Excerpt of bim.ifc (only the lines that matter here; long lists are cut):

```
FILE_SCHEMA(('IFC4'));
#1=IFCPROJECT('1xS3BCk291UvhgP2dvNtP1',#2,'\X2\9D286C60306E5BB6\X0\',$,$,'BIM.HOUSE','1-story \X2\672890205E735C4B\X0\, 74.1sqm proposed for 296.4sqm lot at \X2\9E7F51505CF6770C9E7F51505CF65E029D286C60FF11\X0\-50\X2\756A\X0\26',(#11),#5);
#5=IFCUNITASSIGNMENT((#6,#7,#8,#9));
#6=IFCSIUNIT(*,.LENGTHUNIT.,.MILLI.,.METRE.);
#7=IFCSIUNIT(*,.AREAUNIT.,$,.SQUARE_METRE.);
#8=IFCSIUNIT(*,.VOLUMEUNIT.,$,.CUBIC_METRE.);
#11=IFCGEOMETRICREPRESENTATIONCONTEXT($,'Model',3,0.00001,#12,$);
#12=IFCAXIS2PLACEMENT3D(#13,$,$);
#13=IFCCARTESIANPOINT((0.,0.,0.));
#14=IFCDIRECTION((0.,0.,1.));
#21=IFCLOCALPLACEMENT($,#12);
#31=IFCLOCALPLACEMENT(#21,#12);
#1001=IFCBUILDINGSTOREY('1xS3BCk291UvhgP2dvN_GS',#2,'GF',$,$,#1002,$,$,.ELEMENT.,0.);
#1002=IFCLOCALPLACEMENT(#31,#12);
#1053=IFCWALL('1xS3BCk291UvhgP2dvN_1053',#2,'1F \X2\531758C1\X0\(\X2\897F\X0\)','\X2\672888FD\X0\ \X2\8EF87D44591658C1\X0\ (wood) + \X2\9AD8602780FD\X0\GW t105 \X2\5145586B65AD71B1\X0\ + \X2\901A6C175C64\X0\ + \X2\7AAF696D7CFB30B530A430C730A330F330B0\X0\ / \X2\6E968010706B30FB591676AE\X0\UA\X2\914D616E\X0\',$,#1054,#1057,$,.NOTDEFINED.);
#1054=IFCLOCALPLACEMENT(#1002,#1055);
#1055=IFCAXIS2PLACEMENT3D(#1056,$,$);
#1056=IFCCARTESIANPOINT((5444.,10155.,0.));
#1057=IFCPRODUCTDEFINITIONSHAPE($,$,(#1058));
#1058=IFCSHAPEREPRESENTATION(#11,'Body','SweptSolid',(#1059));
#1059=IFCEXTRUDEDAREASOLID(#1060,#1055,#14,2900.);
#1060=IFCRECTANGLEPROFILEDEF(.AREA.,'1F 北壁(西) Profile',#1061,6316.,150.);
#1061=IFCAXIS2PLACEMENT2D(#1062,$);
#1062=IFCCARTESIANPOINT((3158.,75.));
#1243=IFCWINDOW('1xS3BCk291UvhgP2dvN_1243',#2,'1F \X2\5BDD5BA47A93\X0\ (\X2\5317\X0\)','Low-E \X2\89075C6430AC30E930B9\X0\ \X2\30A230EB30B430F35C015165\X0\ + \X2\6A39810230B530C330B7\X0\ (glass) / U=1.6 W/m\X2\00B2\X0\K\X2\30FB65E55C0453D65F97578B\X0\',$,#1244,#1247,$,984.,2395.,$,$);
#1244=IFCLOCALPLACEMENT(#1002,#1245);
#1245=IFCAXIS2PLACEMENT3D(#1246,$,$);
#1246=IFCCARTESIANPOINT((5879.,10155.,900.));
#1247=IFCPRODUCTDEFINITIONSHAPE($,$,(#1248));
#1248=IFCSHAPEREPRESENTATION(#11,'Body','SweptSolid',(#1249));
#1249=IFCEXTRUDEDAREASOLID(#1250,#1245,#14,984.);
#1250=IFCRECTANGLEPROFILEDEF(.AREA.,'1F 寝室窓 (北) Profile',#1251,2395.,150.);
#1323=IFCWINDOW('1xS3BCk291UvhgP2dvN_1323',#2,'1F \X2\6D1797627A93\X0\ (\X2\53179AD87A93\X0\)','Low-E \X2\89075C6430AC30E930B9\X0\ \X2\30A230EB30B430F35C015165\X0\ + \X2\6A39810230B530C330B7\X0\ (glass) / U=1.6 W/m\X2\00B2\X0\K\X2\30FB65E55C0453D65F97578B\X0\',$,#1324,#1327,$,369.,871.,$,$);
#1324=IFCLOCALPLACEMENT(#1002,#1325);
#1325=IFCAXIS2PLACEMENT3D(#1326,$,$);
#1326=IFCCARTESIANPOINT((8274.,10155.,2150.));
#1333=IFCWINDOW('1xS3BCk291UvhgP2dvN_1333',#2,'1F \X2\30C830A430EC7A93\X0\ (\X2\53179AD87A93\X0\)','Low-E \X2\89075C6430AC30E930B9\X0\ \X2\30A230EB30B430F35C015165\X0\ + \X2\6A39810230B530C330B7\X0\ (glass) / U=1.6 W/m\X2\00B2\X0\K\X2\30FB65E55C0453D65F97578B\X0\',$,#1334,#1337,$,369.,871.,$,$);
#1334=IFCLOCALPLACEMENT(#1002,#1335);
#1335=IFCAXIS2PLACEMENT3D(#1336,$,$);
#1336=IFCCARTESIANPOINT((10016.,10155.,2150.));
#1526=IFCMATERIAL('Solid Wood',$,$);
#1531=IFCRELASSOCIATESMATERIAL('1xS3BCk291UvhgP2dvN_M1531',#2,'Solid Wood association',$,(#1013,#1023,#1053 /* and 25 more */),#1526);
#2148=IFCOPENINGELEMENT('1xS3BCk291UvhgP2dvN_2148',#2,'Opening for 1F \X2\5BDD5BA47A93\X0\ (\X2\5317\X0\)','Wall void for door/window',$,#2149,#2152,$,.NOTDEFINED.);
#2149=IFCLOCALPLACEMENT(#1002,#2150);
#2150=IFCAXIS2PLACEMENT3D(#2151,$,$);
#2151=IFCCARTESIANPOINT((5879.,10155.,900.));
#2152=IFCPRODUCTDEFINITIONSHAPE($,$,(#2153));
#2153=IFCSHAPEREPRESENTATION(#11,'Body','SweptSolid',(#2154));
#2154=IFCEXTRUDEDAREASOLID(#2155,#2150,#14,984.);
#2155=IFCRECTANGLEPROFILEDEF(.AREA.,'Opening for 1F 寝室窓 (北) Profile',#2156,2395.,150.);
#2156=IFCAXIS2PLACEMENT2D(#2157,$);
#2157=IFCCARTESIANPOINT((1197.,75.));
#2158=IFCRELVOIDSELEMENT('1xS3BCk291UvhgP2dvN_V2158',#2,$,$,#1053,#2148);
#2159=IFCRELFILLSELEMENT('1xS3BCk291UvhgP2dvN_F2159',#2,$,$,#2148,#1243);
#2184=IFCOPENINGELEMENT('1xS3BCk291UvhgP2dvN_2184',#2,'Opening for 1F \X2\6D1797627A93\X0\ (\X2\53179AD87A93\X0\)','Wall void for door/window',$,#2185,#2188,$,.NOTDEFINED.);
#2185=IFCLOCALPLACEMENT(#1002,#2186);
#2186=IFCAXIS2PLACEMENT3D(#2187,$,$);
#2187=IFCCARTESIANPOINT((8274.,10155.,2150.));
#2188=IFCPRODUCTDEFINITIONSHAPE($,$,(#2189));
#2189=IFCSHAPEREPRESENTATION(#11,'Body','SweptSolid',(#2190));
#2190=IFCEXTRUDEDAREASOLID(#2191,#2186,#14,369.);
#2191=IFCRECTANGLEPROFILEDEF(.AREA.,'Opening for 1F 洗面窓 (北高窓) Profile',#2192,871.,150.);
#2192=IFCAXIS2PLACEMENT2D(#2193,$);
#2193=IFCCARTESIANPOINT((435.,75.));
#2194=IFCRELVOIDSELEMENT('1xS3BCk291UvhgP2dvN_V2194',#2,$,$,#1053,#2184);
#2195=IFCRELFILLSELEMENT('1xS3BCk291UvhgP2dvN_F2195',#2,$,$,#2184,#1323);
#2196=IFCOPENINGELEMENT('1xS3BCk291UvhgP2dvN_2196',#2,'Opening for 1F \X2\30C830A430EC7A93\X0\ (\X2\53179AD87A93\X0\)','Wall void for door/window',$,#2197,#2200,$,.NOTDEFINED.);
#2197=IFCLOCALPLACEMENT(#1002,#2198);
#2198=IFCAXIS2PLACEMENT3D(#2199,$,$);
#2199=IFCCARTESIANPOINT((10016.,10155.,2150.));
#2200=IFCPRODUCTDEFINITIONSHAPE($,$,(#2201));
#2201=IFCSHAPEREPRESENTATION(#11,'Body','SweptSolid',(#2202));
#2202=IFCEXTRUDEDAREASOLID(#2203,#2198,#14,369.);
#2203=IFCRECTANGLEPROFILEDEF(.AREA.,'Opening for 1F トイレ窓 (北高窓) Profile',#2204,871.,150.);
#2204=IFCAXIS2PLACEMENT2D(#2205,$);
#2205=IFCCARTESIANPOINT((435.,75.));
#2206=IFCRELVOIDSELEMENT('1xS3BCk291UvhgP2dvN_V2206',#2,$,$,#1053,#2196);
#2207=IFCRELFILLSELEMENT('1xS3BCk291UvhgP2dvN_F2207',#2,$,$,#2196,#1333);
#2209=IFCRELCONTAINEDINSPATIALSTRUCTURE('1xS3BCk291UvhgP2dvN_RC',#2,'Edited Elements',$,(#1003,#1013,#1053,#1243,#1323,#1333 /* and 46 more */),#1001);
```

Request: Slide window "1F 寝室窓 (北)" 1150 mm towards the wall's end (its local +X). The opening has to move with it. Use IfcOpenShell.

```python
import ifcopenshell
import ifcopenshell.api.geometry
import ifcopenshell.util.placement
import ifcopenshell.util.unit

model = ifcopenshell.open("bim.ifc")
unit_scale = ifcopenshell.util.unit.calculate_unit_scale(model)

window = model.by_guid("1xS3BCk291UvhgP2dvN_1243")
opening = window.FillsVoids[0].RelatingOpeningElement
wall = opening.VoidsElements[0].RelatingBuildingElement

wall_matrix = ifcopenshell.util.placement.get_local_placement(wall.ObjectPlacement)
shift = wall_matrix[:3, 0] * 1.15 / unit_scale
before = ifcopenshell.util.placement.get_local_placement(window.ObjectPlacement)[:3, 3].copy()

# The window is not placed relative to its opening, so move both.
for product in (opening, window):
    matrix = ifcopenshell.util.placement.get_local_placement(product.ObjectPlacement)
    matrix[:3, 3] += shift
    ifcopenshell.api.geometry.edit_object_placement(model, product=product, matrix=matrix, is_si=False)

after = ifcopenshell.util.placement.get_local_placement(window.ObjectPlacement)[:3, 3]
print("window moved by", (after - before).round(3) + 0.0)

model.write("bim_edited.ifc")
```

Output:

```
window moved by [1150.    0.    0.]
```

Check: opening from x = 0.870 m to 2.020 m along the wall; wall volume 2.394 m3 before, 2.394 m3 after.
